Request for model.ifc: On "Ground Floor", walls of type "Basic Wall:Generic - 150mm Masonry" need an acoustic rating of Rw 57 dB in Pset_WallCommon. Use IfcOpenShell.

First a look at what the model holds.

```python
import ifcopenshell
import ifcopenshell.util.element

model = ifcopenshell.open("model.ifc")
print(model.schema)
storey = next(s for s in model.by_type("IfcBuildingStorey") if s.Name == "Ground Floor")
walls = [e for e in ifcopenshell.util.element.get_decomposition(storey) if e.is_a("IfcWall")]
seen = {}
for e in walls:
    element_type = ifcopenshell.util.element.get_type(e)
    key = (element_type.Name if element_type != e and element_type else None, ifcopenshell.util.element.get_pset(e, "Pset_WallCommon", "AcousticRating"))
    seen[key] = seen.get(key, 0) + 1
for (name, value), count in sorted(seen.items(), key=str):
    print(count, "x", name, "|", value)
```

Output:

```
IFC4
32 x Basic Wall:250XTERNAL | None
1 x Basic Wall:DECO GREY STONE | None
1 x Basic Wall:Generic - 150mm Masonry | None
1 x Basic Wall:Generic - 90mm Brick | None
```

```python
import ifcopenshell
import ifcopenshell.api.pset
import ifcopenshell.util.element

model = ifcopenshell.open("model.ifc")

storey = next(s for s in model.by_type("IfcBuildingStorey") if s.Name == "Ground Floor")
walls = [e for e in ifcopenshell.util.element.get_decomposition(storey) if e.is_a("IfcWall")]

count = 0
for e in walls:
    element_type = ifcopenshell.util.element.get_type(e)
    if element_type in (None, e) or element_type.Name != "Basic Wall:Generic - 150mm Masonry":
        continue
    # add_pset returns the element's existing set when there is one.
    pset = ifcopenshell.api.pset.add_pset(model, product=e, name="Pset_WallCommon")
    ifcopenshell.api.pset.edit_pset(model, pset=pset, properties={"AcousticRating": "Rw 57 dB"})
    count += 1

print(count, "walls updated")

model.write("model_v2.ifc")
```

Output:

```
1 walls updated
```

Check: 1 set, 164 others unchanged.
